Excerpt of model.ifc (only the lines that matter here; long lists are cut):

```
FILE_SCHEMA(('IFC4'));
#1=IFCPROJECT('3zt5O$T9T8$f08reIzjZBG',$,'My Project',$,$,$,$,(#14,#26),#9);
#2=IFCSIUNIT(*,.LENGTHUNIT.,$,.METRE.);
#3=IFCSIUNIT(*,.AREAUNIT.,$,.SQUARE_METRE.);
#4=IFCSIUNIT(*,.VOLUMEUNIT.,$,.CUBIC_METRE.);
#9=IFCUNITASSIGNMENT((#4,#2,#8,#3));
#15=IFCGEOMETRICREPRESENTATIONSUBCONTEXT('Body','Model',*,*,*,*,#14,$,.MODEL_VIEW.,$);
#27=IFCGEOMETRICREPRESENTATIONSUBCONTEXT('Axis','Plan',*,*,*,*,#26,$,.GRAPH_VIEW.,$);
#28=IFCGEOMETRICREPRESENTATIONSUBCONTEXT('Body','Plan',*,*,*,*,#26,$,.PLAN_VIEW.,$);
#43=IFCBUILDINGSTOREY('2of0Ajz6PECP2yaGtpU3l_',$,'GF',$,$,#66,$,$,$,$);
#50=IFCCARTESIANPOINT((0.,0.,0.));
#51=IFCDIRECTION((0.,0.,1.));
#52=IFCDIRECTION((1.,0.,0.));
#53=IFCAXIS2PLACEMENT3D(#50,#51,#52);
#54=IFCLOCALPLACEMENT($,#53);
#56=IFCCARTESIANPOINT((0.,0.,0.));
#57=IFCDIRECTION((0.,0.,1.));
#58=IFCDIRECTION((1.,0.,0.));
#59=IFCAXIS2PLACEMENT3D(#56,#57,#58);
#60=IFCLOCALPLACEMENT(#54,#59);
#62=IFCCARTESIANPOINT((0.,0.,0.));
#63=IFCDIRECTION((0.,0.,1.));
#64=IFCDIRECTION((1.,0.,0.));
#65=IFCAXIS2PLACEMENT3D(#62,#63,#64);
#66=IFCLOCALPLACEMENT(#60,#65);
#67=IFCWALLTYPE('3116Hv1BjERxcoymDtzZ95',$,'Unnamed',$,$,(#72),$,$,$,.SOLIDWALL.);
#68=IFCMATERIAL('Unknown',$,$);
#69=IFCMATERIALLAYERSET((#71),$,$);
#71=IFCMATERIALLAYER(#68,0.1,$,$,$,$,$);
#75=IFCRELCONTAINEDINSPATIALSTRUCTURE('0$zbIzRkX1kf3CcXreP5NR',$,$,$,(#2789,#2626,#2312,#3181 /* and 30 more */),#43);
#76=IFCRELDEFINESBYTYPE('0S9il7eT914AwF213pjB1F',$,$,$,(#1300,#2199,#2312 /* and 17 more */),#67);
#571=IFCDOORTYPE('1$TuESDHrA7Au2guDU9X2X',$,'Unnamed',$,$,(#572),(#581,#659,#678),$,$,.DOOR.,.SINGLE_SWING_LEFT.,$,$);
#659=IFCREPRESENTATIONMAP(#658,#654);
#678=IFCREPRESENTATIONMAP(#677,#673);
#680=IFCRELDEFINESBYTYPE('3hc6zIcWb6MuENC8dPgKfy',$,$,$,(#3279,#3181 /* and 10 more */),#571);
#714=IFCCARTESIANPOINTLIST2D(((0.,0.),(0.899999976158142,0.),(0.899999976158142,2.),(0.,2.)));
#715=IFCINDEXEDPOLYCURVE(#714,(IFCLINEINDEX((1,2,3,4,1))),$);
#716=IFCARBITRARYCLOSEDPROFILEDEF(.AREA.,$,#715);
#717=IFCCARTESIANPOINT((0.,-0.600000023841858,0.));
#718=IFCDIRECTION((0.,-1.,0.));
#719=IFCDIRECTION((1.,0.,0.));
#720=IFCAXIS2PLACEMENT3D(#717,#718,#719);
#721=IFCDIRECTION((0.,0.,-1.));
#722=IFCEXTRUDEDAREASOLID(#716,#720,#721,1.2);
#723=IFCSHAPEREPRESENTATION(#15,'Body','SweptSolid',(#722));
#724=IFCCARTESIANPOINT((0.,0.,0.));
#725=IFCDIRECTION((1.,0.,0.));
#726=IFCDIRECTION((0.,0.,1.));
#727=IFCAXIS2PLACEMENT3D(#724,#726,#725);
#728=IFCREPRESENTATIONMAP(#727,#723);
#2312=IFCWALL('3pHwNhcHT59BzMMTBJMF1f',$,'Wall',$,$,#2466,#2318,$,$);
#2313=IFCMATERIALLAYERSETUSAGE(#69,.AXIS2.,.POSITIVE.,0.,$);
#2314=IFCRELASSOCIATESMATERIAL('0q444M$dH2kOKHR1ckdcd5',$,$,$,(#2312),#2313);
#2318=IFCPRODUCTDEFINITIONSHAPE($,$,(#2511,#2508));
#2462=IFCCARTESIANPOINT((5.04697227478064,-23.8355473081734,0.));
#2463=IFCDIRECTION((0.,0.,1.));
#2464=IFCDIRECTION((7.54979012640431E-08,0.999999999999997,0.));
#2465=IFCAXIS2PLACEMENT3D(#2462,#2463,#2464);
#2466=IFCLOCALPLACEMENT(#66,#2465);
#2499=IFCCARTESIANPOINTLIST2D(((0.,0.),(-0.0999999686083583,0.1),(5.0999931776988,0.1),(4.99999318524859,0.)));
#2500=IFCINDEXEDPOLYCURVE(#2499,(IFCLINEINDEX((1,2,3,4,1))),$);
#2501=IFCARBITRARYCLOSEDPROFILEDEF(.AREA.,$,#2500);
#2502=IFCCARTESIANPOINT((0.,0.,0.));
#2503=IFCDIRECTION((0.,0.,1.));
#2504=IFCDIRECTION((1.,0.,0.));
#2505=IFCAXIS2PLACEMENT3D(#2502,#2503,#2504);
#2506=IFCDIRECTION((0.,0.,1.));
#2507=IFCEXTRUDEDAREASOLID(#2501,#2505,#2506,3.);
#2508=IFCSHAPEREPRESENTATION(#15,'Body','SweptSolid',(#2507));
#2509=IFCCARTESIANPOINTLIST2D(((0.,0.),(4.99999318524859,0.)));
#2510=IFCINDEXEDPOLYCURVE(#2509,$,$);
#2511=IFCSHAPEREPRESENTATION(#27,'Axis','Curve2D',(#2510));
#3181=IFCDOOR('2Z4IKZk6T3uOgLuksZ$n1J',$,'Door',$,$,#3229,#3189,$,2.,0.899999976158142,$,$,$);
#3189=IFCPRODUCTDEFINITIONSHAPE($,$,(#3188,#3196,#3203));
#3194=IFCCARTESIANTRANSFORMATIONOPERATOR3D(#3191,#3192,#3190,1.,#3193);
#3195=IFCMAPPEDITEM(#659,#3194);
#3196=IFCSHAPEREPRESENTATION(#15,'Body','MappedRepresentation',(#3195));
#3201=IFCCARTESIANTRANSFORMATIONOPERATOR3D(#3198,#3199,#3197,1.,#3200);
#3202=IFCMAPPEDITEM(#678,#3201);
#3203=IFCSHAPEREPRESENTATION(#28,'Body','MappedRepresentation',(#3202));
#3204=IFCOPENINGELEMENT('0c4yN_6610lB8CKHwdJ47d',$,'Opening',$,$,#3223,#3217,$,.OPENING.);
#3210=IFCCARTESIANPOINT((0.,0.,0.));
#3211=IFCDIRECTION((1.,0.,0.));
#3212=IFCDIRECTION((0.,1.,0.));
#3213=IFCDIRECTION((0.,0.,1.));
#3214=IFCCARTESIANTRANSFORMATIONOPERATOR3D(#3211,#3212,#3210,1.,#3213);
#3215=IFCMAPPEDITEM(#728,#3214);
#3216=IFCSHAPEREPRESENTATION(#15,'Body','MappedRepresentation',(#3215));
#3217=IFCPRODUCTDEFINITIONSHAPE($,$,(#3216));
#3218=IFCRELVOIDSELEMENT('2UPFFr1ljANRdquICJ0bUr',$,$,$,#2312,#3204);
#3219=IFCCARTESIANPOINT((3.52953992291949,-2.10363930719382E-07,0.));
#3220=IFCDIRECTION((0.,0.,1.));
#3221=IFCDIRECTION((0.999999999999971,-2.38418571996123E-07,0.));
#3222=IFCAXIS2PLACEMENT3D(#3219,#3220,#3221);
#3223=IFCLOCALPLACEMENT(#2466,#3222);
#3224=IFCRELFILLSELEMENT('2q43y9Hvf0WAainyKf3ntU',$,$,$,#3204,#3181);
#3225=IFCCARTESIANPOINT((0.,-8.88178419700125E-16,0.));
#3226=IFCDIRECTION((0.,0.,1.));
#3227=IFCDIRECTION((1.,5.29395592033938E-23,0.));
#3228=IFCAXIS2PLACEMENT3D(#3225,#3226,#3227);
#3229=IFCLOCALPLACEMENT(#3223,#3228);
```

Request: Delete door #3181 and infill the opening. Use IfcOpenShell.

```python
import ifcopenshell
import ifcopenshell.api.feature
import ifcopenshell.api.root
import ifcopenshell.geom
import ifcopenshell.util.shape

model = ifcopenshell.open("model.ifc")
settings = ifcopenshell.geom.settings()


def volume(element):
    """Net volume in cubic metres, openings subtracted."""
    shape = ifcopenshell.geom.create_shape(settings, element)
    return ifcopenshell.util.shape.get_volume(shape.geometry)


door = model.by_guid("2Z4IKZk6T3uOgLuksZ$n1J")
opening = door.FillsVoids[0].RelatingOpeningElement
wall = opening.VoidsElements[0].RelatingBuildingElement
before = volume(wall)

ifcopenshell.api.root.remove_product(model, product=door)
ifcopenshell.api.feature.remove_feature(model, feature=opening)

after = volume(wall)

print(f"wall volume {before:.3f} -> {after:.3f} m3")

model.write("model_rev.ifc")
```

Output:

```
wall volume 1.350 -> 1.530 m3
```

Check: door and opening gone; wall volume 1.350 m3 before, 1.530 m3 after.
